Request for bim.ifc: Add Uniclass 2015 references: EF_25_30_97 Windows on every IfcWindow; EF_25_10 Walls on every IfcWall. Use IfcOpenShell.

First a look at what the model holds.

```python
import ifcopenshell

model = ifcopenshell.open("bim.ifc")
print(model.schema)
print("classifications:", [c.Name for c in model.by_type("IfcClassification")])
for ifc_class in ("IfcDoor", "IfcRoof", "IfcStair", "IfcWall", "IfcWindow"):
    print(ifc_class, len(model.by_type(ifc_class)))
```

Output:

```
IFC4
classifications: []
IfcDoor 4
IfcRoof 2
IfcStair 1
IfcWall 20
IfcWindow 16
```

```python
import ifcopenshell
import ifcopenshell.api.classification

model = ifcopenshell.open("bim.ifc")

system = ifcopenshell.api.classification.add_classification(model, classification="Uniclass 2015")

codes = {
    "IfcWindow": ("EF_25_30_97", "Windows"),
    "IfcWall": ("EF_25_10", "Walls"),
}
for ifc_class, (code, name) in codes.items():
    products = model.by_type(ifc_class)
    ifcopenshell.api.classification.add_reference(
        model, products=products, classification=system, identification=code, name=name
    )
    print(code, len(products))

model.write("bim_rev.ifc")
```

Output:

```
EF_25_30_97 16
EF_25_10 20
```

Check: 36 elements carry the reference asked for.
